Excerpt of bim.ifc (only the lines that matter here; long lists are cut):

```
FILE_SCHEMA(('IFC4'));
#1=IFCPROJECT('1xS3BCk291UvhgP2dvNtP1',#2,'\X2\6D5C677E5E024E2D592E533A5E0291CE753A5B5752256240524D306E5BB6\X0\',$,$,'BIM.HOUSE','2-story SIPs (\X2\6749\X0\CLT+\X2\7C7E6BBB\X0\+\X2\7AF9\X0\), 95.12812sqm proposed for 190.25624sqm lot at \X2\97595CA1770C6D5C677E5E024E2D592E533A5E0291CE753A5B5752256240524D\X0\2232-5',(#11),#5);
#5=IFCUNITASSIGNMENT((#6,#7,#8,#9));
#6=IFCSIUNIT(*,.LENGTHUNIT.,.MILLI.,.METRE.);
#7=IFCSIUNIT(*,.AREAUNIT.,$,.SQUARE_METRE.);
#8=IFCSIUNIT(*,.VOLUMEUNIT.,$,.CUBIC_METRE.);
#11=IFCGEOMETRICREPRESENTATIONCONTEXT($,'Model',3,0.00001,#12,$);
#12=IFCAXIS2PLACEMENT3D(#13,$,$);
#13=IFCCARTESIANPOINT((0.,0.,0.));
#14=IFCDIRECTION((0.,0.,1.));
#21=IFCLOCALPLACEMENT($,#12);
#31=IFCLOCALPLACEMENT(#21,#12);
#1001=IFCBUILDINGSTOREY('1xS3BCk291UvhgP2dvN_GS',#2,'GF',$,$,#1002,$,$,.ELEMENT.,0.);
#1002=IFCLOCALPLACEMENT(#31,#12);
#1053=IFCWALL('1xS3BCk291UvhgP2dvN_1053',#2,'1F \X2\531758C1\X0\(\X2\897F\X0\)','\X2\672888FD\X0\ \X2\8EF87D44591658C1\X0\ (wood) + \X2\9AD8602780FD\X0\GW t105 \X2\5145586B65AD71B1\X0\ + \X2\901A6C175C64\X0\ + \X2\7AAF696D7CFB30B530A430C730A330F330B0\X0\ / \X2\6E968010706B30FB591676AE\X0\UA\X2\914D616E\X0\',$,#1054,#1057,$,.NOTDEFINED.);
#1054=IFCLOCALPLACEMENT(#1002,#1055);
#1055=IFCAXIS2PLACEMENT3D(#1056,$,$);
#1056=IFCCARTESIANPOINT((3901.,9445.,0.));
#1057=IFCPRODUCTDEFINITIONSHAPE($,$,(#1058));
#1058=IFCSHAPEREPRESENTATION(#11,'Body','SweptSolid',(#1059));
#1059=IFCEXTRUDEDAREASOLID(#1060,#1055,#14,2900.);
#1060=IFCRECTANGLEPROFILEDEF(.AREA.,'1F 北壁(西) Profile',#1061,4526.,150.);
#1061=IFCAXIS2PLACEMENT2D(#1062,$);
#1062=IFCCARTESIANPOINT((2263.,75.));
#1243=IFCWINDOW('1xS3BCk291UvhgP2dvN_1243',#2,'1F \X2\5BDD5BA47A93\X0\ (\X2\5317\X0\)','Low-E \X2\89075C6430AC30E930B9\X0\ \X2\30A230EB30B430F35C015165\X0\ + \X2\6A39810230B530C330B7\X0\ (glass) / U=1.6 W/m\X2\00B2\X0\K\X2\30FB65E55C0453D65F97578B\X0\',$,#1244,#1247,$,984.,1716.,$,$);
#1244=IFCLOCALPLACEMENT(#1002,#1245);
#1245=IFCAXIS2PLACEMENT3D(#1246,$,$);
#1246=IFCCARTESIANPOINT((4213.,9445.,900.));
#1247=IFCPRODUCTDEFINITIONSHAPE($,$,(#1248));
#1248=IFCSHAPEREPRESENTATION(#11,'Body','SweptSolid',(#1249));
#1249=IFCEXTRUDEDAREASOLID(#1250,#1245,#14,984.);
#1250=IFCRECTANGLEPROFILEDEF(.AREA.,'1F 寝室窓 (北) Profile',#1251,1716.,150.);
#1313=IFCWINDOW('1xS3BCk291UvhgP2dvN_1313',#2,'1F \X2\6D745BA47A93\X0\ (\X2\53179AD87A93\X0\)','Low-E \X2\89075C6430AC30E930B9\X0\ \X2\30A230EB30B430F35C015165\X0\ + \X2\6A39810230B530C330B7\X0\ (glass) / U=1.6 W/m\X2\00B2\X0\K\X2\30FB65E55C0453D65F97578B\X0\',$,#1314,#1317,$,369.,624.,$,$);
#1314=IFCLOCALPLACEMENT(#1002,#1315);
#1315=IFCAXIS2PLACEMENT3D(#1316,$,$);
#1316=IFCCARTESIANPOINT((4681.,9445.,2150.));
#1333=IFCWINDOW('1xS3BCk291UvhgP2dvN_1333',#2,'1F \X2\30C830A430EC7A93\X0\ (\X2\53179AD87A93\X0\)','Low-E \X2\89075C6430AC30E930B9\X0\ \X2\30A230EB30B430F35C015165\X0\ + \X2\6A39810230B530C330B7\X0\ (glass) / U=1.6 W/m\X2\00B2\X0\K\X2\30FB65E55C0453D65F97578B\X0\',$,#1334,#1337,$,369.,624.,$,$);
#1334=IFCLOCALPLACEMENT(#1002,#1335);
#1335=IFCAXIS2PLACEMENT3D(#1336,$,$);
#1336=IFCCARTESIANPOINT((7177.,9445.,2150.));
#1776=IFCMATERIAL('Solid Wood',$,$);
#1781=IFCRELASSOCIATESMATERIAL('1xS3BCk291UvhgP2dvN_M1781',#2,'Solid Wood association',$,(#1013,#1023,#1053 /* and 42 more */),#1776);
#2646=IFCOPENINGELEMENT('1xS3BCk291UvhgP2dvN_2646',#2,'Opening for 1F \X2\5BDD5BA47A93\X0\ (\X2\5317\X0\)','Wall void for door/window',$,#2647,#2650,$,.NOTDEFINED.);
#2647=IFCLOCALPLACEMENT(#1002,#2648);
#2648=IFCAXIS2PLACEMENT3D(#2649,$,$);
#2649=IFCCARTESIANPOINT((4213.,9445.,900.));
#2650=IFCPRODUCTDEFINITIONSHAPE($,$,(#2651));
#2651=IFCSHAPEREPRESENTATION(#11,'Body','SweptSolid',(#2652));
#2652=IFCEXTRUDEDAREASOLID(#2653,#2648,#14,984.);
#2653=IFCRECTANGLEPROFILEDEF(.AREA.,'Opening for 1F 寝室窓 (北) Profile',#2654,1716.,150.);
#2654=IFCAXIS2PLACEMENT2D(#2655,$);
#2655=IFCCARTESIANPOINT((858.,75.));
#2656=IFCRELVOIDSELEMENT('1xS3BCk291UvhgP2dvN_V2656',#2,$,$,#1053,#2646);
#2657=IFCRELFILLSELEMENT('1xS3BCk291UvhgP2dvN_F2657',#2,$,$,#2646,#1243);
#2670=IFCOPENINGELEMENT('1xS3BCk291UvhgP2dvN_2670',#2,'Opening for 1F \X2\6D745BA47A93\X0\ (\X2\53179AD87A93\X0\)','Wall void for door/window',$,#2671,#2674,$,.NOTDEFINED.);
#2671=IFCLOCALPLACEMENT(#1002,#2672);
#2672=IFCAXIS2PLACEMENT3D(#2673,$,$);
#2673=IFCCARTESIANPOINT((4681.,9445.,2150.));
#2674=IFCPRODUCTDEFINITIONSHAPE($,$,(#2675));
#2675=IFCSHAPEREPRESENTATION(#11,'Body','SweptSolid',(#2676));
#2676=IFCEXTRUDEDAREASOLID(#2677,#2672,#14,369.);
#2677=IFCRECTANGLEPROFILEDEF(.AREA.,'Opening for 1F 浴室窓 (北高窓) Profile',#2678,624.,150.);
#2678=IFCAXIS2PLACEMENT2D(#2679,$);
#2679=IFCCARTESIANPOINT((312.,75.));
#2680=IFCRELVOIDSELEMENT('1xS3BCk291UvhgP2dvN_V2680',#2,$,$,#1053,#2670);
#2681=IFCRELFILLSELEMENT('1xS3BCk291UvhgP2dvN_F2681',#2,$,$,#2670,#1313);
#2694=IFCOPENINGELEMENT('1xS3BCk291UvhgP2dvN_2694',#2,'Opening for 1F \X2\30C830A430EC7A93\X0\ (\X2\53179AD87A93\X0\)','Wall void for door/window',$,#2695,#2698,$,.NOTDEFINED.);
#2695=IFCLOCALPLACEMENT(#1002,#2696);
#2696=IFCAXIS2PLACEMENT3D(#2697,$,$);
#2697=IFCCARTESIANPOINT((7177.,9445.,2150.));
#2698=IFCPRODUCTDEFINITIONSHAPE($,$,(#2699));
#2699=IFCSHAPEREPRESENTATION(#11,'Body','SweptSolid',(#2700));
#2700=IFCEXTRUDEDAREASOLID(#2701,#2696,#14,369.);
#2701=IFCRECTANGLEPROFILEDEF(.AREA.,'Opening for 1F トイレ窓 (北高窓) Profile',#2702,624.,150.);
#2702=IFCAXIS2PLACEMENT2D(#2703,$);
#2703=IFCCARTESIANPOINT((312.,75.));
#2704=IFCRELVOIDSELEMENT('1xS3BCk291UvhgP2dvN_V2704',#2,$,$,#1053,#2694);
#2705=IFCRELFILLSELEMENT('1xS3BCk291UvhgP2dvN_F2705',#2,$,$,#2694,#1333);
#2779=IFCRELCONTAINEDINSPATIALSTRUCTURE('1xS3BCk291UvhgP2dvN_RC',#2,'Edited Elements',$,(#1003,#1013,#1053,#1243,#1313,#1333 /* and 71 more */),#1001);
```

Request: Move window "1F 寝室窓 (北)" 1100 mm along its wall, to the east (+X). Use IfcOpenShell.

```python
import ifcopenshell
import ifcopenshell.api.geometry
import ifcopenshell.util.placement
import ifcopenshell.util.unit

model = ifcopenshell.open("bim.ifc")
unit_scale = ifcopenshell.util.unit.calculate_unit_scale(model)

window = model.by_id(1243)
opening = window.FillsVoids[0].RelatingOpeningElement
wall = opening.VoidsElements[0].RelatingBuildingElement

wall_matrix = ifcopenshell.util.placement.get_local_placement(wall.ObjectPlacement)
shift = wall_matrix[:3, 0] * 1.1 / unit_scale
before = ifcopenshell.util.placement.get_local_placement(window.ObjectPlacement)[:3, 3].copy()

# The window is not placed relative to its opening, so move both.
for product in (opening, window):
    matrix = ifcopenshell.util.placement.get_local_placement(product.ObjectPlacement)
    matrix[:3, 3] += shift
    ifcopenshell.api.geometry.edit_object_placement(model, product=product, matrix=matrix, is_si=False)

after = ifcopenshell.util.placement.get_local_placement(window.ObjectPlacement)[:3, 3]
print("window moved by", (after - before).round(3) + 0.0)

model.write("bim_edited.ifc")
```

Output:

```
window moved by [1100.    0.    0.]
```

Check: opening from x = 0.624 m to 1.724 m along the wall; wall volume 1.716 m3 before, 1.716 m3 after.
